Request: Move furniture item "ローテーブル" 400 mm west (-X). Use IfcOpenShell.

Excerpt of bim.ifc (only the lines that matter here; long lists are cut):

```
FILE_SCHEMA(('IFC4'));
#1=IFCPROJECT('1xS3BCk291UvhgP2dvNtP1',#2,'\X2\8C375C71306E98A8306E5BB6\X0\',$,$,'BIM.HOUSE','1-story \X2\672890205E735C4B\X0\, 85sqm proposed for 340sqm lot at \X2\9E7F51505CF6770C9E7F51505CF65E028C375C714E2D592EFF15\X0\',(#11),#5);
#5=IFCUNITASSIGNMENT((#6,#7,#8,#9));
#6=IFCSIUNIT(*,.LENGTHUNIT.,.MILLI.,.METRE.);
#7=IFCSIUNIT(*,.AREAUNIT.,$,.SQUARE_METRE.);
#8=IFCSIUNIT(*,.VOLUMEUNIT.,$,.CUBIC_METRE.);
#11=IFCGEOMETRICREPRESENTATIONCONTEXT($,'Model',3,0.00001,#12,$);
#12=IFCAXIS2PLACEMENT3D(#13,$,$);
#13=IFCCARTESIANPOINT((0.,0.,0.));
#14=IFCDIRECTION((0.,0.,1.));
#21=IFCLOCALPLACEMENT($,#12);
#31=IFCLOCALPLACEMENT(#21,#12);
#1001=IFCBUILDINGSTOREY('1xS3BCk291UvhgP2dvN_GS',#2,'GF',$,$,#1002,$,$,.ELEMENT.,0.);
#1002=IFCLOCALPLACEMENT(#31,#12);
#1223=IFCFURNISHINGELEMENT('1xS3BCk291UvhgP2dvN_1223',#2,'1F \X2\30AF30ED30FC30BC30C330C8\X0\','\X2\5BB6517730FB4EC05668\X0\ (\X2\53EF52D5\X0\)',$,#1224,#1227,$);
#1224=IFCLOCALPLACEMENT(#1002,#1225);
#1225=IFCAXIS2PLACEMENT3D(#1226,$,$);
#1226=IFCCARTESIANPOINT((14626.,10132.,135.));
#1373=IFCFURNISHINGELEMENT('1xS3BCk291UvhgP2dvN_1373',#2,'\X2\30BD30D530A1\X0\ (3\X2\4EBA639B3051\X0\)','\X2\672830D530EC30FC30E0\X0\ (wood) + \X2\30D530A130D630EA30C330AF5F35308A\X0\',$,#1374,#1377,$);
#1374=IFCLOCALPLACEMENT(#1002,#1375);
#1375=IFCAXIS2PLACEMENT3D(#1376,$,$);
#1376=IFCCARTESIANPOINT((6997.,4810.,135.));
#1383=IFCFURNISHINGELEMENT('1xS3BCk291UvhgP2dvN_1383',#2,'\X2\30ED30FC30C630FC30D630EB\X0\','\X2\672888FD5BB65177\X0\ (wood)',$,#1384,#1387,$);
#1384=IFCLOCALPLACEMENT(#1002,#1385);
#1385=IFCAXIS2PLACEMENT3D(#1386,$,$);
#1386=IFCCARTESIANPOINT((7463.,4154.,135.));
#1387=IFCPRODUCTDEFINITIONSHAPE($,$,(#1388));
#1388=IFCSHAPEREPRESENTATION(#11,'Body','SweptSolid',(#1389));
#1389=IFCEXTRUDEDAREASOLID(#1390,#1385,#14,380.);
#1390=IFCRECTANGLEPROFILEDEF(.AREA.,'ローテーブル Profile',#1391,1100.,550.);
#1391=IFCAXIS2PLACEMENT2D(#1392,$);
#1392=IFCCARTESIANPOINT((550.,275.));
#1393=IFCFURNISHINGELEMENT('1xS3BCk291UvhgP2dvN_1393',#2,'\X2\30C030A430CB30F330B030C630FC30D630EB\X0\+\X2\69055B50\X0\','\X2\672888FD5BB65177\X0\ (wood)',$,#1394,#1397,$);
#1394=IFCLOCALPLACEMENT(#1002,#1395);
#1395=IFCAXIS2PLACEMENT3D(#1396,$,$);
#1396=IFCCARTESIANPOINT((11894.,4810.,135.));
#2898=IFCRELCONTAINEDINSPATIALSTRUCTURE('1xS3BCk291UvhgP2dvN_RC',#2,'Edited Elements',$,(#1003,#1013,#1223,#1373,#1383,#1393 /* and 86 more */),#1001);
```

```python
import ifcopenshell
import ifcopenshell.api.geometry
import ifcopenshell.util.placement
import ifcopenshell.util.unit

model = ifcopenshell.open("bim.ifc")
unit_scale = ifcopenshell.util.unit.calculate_unit_scale(model)

item = model.by_id(1383)
matrix = ifcopenshell.util.placement.get_local_placement(item.ObjectPlacement)
matrix[0, 3] -= 0.4 / unit_scale
ifcopenshell.api.geometry.edit_object_placement(model, product=item, matrix=matrix, is_si=False)

print(ifcopenshell.util.placement.get_local_placement(item.ObjectPlacement).round(3) + 0.0)

model.write("bim_edited.ifc")
```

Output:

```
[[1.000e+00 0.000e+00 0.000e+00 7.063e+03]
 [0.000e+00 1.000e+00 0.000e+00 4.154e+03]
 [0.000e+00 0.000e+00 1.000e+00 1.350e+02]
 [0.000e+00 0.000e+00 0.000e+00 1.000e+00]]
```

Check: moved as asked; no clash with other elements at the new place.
